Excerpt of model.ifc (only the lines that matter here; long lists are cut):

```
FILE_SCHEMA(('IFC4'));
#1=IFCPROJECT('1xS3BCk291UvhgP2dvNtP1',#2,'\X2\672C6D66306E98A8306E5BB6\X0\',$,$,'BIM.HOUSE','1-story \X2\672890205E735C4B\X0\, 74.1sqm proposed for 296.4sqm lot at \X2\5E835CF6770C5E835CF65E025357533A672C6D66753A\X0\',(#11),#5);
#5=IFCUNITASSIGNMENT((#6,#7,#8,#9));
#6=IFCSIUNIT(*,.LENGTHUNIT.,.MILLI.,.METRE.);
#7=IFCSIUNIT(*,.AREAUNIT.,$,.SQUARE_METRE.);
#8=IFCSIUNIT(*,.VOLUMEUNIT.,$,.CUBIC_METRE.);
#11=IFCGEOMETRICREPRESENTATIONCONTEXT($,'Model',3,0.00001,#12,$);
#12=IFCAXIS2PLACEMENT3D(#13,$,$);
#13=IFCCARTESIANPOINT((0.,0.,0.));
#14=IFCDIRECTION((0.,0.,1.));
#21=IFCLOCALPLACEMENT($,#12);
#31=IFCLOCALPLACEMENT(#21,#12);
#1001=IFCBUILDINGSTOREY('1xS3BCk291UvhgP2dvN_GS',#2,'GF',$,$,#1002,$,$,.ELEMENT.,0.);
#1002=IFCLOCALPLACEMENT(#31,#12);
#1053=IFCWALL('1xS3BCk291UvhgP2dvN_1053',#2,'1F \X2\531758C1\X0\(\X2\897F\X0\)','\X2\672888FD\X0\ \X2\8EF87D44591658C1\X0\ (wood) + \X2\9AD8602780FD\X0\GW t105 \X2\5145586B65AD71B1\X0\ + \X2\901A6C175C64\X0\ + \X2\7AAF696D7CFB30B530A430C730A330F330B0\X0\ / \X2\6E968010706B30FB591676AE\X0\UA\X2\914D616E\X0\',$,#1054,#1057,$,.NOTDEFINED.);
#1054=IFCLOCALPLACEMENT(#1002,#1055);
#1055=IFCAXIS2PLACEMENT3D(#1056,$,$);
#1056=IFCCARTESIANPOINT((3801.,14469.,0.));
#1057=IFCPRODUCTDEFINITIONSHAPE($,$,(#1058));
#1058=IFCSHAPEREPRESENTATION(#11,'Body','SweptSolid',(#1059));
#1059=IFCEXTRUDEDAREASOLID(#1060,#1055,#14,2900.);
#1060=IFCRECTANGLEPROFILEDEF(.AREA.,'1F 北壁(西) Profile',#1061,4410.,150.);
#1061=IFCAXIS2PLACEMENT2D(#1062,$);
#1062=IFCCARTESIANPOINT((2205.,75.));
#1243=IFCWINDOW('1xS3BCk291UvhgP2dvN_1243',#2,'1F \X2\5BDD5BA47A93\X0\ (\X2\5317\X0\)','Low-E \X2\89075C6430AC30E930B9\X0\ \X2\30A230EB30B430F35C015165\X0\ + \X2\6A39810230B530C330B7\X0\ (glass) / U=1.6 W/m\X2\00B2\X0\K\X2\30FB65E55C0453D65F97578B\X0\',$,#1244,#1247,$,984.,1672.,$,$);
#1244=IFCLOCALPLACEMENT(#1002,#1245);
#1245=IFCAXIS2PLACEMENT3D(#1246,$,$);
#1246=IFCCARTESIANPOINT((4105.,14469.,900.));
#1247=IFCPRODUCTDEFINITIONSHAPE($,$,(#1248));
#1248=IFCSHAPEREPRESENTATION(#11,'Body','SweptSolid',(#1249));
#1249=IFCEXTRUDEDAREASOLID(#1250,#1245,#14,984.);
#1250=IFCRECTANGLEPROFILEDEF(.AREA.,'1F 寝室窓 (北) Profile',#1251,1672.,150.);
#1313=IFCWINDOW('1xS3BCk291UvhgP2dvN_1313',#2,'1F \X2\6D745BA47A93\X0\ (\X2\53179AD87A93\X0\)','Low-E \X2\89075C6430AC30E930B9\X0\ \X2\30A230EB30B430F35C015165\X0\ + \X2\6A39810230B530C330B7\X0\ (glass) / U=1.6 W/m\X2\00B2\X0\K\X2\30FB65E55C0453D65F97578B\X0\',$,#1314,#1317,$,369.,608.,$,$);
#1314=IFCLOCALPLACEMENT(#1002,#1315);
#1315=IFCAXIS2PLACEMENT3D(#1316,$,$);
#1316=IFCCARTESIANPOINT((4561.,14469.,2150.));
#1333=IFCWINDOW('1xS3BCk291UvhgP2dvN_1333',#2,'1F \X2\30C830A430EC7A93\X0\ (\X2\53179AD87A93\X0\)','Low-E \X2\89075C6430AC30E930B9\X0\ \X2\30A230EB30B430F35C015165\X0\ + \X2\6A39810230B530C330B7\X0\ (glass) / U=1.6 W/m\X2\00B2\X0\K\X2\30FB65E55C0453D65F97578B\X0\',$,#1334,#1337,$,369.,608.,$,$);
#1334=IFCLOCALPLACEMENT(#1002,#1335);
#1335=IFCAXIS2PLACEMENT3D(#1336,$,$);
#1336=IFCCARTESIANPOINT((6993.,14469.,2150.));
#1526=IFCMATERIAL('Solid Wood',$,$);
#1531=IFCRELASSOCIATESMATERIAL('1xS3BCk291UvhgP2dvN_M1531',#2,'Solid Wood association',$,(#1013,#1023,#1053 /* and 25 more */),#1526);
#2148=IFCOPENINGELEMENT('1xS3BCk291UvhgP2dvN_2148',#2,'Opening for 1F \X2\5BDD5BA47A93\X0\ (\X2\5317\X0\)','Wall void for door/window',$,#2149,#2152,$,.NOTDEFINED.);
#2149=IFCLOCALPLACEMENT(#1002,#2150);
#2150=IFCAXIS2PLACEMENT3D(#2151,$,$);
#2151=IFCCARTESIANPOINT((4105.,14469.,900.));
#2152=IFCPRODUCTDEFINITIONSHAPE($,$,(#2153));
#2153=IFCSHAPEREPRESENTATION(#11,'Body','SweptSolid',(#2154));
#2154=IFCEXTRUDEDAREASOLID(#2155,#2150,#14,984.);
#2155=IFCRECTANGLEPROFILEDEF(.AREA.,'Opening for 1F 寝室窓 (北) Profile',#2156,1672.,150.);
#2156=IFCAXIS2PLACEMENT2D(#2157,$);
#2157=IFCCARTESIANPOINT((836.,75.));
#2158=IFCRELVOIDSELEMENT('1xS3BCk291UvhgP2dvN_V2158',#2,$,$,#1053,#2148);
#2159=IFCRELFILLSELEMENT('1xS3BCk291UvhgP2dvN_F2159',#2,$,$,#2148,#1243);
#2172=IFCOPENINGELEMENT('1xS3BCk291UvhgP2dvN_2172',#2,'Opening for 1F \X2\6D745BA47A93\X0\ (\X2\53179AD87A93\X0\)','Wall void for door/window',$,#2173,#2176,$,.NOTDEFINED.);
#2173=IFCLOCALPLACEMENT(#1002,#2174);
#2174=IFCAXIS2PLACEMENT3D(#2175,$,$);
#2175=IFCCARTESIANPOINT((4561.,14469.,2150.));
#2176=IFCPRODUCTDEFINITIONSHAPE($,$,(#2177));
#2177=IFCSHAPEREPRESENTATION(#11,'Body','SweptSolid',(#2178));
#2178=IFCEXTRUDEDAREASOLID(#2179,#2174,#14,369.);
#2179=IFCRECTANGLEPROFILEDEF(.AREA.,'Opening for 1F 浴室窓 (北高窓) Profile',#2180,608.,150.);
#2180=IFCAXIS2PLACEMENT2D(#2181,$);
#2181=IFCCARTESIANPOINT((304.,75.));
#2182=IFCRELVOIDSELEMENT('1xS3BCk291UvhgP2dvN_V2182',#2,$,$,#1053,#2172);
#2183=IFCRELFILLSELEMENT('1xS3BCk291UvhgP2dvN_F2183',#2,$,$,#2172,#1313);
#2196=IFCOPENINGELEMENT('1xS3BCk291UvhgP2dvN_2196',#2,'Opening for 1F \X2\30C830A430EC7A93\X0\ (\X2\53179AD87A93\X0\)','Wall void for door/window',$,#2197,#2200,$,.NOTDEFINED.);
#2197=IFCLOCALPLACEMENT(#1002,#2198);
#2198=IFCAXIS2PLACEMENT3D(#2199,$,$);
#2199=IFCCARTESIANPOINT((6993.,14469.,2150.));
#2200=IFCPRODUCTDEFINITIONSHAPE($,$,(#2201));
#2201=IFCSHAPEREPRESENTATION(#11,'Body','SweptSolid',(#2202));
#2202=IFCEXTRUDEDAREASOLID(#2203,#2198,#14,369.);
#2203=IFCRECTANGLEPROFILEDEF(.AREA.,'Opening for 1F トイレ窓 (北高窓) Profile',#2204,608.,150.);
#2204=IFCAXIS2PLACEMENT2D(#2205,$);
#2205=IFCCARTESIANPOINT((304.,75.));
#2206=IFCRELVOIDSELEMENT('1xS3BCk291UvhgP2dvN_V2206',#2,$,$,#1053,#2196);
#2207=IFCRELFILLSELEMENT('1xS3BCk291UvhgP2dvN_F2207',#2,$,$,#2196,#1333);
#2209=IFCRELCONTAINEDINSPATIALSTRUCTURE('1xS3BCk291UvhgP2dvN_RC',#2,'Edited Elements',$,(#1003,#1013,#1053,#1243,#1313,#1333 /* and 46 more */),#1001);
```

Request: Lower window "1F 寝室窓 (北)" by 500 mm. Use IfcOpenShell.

```python
import numpy as np
import ifcopenshell
import ifcopenshell.api.geometry
import ifcopenshell.util.placement
import ifcopenshell.util.unit

model = ifcopenshell.open("model.ifc")
unit_scale = ifcopenshell.util.unit.calculate_unit_scale(model)

window = model.by_id(1243)
opening = window.FillsVoids[0].RelatingOpeningElement
dz = -0.5 / unit_scale

shift = np.array([0.0, 0.0, dz])
# The window is not placed relative to its opening, so move both.
for product in (opening, window):
    matrix = ifcopenshell.util.placement.get_local_placement(product.ObjectPlacement)
    matrix[:3, 3] += shift
    ifcopenshell.api.geometry.edit_object_placement(model, product=product, matrix=matrix, is_si=False)

print(f"moved by {dz * unit_scale:+.3f} m")

model.write("model_v2.ifc")
```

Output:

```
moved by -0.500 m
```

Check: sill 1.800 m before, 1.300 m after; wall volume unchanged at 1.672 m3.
